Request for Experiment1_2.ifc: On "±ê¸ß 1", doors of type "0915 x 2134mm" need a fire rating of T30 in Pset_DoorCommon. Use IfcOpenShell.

First a look at what the model holds.

```python
import ifcopenshell
import ifcopenshell.util.element

model = ifcopenshell.open("Experiment1_2.ifc")
print(model.schema)
storey = next(s for s in model.by_type("IfcBuildingStorey") if s.Name == "±ê¸ß 1")
doors = [e for e in ifcopenshell.util.element.get_decomposition(storey) if e.is_a("IfcDoor")]
seen = {}
for e in doors:
    element_type = ifcopenshell.util.element.get_type(e)
    key = (element_type.Name if element_type != e and element_type else None, ifcopenshell.util.element.get_pset(e, "Pset_DoorCommon", "FireRating"))
    seen[key] = seen.get(key, 0) + 1
for (name, value), count in sorted(seen.items(), key=str):
    print(count, "x", name, "|", value)
```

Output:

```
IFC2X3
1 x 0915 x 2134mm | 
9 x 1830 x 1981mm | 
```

```python
import ifcopenshell
import ifcopenshell.api.pset
import ifcopenshell.util.element

model = ifcopenshell.open("Experiment1_2.ifc")

storey = next(s for s in model.by_type("IfcBuildingStorey") if s.Name == "±ê¸ß 1")
doors = [e for e in ifcopenshell.util.element.get_decomposition(storey) if e.is_a("IfcDoor")]

count = 0
for e in doors:
    element_type = ifcopenshell.util.element.get_type(e)
    if element_type in (None, e) or element_type.Name != "0915 x 2134mm":
        continue
    # add_pset returns the element's existing set when there is one.
    pset = ifcopenshell.api.pset.add_pset(model, product=e, name="Pset_DoorCommon")
    ifcopenshell.api.pset.edit_pset(model, pset=pset, properties={"FireRating": "T30"})
    count += 1

print(count, "doors updated")

model.write("Experiment1_2_v2.ifc")
```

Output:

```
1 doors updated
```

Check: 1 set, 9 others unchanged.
